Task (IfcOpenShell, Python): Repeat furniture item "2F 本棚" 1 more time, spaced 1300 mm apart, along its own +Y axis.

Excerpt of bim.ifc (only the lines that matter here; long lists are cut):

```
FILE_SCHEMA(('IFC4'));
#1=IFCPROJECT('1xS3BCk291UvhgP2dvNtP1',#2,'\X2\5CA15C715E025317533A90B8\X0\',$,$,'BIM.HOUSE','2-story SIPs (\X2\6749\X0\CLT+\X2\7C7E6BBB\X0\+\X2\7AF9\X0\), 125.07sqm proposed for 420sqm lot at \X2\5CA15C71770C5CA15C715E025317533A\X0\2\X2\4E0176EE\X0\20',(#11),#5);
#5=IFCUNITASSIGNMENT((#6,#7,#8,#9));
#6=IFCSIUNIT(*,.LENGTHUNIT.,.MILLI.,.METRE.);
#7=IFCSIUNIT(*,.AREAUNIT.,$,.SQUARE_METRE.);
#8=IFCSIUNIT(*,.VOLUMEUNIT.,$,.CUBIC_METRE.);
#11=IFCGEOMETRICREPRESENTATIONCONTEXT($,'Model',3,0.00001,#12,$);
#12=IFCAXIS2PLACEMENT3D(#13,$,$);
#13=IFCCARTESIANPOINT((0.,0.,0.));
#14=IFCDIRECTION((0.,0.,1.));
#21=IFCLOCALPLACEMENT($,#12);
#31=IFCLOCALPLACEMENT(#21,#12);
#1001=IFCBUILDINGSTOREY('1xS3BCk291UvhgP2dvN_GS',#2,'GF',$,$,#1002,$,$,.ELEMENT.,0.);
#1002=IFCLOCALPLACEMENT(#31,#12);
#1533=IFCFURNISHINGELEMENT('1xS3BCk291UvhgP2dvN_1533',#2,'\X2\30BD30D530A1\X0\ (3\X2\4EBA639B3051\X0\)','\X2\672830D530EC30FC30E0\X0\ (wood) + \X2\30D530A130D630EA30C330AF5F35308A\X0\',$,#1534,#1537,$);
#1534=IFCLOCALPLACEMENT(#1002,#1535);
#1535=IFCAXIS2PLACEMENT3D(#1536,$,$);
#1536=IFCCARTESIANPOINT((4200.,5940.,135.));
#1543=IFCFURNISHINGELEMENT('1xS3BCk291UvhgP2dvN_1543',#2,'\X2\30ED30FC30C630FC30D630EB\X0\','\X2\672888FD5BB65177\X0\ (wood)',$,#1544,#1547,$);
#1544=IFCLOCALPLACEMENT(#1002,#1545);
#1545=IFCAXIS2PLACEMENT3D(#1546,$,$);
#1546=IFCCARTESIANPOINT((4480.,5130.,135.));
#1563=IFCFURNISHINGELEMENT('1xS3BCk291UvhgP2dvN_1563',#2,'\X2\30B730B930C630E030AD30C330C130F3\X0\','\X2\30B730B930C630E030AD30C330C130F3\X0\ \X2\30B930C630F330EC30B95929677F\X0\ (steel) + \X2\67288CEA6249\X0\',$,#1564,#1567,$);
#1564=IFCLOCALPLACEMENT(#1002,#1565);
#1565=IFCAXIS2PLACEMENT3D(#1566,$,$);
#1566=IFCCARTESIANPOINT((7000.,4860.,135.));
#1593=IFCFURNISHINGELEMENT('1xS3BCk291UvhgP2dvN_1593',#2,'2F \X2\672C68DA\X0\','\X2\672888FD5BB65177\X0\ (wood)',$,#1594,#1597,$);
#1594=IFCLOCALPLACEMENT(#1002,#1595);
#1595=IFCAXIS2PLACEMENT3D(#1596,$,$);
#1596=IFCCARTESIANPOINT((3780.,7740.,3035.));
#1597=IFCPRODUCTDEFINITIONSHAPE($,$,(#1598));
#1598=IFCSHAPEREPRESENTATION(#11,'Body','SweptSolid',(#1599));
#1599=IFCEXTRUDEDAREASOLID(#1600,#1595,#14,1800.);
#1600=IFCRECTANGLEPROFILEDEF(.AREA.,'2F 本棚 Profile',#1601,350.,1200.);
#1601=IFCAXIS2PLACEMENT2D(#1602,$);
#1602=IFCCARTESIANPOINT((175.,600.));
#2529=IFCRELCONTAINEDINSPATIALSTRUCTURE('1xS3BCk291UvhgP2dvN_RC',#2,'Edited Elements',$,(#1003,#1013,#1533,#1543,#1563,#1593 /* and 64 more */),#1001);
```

```python
import ifcopenshell
import ifcopenshell.api.geometry
import ifcopenshell.api.root
import ifcopenshell.util.element
import ifcopenshell.util.placement
import ifcopenshell.util.unit

model = ifcopenshell.open("bim.ifc")
unit_scale = ifcopenshell.util.unit.calculate_unit_scale(model)


def reuse_history(source, copy):
    """copy_class also copies each property set's owner history, people and application; keep the originals."""
    for rel in copy.IsDefinedBy:
        if rel.is_a("IfcRelDefinesByProperties") and (history := rel.RelatingPropertyDefinition.OwnerHistory):
            rel.RelatingPropertyDefinition.OwnerHistory = source.OwnerHistory
            ifcopenshell.util.element.remove_deep2(model, history)


source = model.by_guid("1xS3BCk291UvhgP2dvN_1593")
base = ifcopenshell.util.placement.get_local_placement(source.ObjectPlacement)
step = base[:3, 1] * 1.3 / unit_scale

for i in range(1, 2):
    copy = ifcopenshell.api.root.copy_class(model, product=source)
    copy.Representation = ifcopenshell.util.element.copy_deep(
        model, source.Representation, exclude=["IfcGeometricRepresentationContext", "IfcRepresentationMap"]
    )
    reuse_history(source, copy)
    matrix = base.copy()
    matrix[:3, 3] += i * step
    print("added at", matrix[:3, 3].round(3) + 0.0)
    ifcopenshell.api.geometry.edit_object_placement(model, product=copy, matrix=matrix, is_si=False)

model.write("bim_updated.ifc")
```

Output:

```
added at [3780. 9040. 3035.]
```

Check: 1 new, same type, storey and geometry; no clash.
